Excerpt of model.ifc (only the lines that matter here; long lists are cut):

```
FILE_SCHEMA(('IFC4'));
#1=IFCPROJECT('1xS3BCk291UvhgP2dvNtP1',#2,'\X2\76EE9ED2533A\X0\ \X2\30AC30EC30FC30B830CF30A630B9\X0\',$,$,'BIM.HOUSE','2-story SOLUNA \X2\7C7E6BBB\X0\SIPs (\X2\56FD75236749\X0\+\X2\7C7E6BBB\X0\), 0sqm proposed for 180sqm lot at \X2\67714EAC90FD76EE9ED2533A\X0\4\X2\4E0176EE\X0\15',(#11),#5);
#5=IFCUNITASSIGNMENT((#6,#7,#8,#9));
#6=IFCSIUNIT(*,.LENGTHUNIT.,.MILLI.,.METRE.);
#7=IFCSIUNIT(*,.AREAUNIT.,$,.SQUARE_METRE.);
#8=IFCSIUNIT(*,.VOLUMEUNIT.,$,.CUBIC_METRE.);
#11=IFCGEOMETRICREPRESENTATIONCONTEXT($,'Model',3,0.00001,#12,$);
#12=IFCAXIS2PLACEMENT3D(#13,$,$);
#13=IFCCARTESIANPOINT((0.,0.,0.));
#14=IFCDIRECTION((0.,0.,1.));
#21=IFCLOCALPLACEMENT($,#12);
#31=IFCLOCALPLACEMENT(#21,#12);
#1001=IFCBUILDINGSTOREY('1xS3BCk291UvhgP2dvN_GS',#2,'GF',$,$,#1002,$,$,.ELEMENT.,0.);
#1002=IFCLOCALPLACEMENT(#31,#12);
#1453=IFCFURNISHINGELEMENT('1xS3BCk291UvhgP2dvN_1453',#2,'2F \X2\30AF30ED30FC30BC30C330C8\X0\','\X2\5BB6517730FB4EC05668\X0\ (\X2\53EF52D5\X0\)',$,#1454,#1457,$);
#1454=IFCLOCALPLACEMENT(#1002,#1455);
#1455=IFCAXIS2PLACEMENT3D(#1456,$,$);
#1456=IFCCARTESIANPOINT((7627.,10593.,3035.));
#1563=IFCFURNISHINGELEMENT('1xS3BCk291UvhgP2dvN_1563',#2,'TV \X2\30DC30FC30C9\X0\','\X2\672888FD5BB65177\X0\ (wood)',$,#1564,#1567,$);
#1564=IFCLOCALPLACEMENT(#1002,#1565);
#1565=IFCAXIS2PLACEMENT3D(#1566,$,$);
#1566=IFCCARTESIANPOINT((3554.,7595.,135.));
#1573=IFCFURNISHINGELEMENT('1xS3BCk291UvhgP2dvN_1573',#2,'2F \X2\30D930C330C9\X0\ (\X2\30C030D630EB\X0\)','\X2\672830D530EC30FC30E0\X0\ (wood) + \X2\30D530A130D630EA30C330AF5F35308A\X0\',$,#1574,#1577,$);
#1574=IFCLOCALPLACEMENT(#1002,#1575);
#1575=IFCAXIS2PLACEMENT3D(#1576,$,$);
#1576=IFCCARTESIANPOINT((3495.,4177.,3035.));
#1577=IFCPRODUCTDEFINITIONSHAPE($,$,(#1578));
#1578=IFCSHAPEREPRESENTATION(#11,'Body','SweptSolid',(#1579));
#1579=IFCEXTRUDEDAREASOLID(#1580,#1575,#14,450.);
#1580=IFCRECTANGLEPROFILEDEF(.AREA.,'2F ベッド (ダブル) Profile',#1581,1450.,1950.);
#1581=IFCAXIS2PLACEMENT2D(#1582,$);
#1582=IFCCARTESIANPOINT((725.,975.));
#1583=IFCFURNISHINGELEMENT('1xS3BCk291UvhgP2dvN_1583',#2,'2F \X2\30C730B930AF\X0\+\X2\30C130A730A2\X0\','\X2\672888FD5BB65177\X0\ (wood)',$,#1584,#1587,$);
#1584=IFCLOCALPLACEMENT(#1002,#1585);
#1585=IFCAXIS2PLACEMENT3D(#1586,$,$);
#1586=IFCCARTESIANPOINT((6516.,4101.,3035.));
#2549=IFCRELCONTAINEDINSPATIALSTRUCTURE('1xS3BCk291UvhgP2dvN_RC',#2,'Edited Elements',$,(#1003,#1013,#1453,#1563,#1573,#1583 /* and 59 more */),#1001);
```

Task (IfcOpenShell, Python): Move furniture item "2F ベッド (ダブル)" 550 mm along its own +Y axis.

```python
import ifcopenshell
import ifcopenshell.api.geometry
import ifcopenshell.util.placement

model = ifcopenshell.open("model.ifc")

item = model.by_guid("1xS3BCk291UvhgP2dvN_1573")
matrix = ifcopenshell.util.placement.get_local_placement(item.ObjectPlacement)
matrix[:3, 3] += matrix[:3, 1] * 550.0
ifcopenshell.api.geometry.edit_object_placement(model, product=item, matrix=matrix, is_si=False)

print(ifcopenshell.util.placement.get_local_placement(item.ObjectPlacement).round(3) + 0.0)

model.write("model_v2.ifc")
```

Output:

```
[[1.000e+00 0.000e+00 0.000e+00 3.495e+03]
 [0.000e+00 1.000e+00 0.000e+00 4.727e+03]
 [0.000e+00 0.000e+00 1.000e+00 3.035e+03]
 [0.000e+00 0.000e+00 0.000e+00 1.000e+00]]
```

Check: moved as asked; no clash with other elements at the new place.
